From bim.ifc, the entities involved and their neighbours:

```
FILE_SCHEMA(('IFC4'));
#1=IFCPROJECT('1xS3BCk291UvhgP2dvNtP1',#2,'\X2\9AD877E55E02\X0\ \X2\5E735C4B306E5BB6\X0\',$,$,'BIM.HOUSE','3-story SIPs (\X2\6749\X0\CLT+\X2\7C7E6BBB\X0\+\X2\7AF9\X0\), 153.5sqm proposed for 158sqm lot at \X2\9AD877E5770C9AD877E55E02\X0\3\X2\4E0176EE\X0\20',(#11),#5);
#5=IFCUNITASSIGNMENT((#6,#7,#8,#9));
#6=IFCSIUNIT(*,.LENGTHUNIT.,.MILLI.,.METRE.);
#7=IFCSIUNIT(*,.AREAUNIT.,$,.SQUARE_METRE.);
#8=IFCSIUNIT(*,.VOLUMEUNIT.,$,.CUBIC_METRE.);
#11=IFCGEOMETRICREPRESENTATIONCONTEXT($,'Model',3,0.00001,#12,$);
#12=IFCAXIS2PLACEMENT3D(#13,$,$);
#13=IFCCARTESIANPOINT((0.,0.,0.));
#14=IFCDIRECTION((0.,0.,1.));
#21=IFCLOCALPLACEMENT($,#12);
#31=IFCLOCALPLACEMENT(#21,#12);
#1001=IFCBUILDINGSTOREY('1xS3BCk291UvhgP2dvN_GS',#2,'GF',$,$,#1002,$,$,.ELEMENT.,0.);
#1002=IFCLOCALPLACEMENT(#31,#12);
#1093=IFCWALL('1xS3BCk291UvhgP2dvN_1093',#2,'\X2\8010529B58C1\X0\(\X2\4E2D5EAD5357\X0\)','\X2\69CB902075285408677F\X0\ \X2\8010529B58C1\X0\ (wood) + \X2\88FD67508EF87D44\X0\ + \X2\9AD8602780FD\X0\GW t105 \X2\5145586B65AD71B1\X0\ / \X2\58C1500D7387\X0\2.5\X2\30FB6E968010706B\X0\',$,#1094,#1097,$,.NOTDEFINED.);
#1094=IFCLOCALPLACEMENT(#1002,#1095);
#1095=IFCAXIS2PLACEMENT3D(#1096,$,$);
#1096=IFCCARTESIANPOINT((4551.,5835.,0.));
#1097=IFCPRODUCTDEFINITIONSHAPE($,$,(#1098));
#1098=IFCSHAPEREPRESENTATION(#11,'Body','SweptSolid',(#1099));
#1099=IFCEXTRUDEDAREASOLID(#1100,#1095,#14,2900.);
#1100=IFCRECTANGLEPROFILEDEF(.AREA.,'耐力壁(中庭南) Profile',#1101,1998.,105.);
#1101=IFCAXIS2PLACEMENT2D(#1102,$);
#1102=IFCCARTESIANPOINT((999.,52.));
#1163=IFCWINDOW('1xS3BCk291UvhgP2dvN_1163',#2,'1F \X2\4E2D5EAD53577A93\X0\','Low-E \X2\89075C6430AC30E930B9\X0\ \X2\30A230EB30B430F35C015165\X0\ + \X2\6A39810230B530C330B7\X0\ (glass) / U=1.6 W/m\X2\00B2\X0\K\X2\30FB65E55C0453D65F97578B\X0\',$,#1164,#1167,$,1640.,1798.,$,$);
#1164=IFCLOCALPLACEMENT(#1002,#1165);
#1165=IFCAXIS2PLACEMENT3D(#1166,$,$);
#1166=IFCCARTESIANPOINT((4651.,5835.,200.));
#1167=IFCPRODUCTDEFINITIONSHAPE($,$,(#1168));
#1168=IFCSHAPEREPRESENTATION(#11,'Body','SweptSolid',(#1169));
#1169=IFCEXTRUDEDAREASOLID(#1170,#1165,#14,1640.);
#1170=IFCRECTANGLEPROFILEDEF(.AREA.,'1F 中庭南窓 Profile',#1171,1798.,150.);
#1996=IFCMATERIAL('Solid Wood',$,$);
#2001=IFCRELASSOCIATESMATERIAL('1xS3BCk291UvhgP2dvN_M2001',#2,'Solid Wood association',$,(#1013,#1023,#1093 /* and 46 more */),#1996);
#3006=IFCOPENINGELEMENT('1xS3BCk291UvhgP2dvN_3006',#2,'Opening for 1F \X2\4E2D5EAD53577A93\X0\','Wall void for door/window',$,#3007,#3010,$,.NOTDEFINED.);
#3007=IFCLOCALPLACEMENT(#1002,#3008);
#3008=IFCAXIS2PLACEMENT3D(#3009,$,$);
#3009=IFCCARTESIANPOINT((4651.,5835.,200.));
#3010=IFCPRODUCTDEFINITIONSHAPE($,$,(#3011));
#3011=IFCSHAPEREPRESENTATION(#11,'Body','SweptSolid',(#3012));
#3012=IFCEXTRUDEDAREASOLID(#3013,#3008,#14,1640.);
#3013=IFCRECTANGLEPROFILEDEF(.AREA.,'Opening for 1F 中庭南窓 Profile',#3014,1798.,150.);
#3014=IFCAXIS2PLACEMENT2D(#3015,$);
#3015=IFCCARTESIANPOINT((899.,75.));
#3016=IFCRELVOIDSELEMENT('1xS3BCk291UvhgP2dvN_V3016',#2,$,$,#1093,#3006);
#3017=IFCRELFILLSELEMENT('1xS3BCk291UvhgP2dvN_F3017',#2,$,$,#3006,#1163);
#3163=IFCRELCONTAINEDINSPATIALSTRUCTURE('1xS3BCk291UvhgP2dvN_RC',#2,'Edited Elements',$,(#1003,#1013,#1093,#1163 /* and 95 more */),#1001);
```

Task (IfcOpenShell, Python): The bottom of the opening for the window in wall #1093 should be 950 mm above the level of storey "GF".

```python
import numpy as np
import ifcopenshell
import ifcopenshell.api.geometry
import ifcopenshell.geom
import ifcopenshell.util.element
import ifcopenshell.util.placement
import ifcopenshell.util.shape
import ifcopenshell.util.unit

model = ifcopenshell.open("bim.ifc")
unit_scale = ifcopenshell.util.unit.calculate_unit_scale(model)

window = model.by_guid("1xS3BCk291UvhgP2dvN_1163")
opening = window.FillsVoids[0].RelatingOpeningElement
storey = ifcopenshell.util.element.get_container(window, ifc_class="IfcBuildingStorey")
level = ifcopenshell.util.placement.get_local_placement(storey.ObjectPlacement)[2, 3]

# The opening's origin need not be at the sill, so measure its lowest point.
shape = ifcopenshell.geom.create_shape(ifcopenshell.geom.settings(), opening)
bottom = ifcopenshell.util.shape.get_shape_bottom_elevation(shape, shape.geometry) / unit_scale
dz = level + 0.95 / unit_scale - bottom

shift = np.array([0.0, 0.0, dz])
# The window is not placed relative to its opening, so move both.
for product in (opening, window):
    matrix = ifcopenshell.util.placement.get_local_placement(product.ObjectPlacement)
    matrix[:3, 3] += shift
    ifcopenshell.api.geometry.edit_object_placement(model, product=product, matrix=matrix, is_si=False)

print(f"moved by {dz * unit_scale:+.3f} m")

model.write("bim_edited.ifc")
```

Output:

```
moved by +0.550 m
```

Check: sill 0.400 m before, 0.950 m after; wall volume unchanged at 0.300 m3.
